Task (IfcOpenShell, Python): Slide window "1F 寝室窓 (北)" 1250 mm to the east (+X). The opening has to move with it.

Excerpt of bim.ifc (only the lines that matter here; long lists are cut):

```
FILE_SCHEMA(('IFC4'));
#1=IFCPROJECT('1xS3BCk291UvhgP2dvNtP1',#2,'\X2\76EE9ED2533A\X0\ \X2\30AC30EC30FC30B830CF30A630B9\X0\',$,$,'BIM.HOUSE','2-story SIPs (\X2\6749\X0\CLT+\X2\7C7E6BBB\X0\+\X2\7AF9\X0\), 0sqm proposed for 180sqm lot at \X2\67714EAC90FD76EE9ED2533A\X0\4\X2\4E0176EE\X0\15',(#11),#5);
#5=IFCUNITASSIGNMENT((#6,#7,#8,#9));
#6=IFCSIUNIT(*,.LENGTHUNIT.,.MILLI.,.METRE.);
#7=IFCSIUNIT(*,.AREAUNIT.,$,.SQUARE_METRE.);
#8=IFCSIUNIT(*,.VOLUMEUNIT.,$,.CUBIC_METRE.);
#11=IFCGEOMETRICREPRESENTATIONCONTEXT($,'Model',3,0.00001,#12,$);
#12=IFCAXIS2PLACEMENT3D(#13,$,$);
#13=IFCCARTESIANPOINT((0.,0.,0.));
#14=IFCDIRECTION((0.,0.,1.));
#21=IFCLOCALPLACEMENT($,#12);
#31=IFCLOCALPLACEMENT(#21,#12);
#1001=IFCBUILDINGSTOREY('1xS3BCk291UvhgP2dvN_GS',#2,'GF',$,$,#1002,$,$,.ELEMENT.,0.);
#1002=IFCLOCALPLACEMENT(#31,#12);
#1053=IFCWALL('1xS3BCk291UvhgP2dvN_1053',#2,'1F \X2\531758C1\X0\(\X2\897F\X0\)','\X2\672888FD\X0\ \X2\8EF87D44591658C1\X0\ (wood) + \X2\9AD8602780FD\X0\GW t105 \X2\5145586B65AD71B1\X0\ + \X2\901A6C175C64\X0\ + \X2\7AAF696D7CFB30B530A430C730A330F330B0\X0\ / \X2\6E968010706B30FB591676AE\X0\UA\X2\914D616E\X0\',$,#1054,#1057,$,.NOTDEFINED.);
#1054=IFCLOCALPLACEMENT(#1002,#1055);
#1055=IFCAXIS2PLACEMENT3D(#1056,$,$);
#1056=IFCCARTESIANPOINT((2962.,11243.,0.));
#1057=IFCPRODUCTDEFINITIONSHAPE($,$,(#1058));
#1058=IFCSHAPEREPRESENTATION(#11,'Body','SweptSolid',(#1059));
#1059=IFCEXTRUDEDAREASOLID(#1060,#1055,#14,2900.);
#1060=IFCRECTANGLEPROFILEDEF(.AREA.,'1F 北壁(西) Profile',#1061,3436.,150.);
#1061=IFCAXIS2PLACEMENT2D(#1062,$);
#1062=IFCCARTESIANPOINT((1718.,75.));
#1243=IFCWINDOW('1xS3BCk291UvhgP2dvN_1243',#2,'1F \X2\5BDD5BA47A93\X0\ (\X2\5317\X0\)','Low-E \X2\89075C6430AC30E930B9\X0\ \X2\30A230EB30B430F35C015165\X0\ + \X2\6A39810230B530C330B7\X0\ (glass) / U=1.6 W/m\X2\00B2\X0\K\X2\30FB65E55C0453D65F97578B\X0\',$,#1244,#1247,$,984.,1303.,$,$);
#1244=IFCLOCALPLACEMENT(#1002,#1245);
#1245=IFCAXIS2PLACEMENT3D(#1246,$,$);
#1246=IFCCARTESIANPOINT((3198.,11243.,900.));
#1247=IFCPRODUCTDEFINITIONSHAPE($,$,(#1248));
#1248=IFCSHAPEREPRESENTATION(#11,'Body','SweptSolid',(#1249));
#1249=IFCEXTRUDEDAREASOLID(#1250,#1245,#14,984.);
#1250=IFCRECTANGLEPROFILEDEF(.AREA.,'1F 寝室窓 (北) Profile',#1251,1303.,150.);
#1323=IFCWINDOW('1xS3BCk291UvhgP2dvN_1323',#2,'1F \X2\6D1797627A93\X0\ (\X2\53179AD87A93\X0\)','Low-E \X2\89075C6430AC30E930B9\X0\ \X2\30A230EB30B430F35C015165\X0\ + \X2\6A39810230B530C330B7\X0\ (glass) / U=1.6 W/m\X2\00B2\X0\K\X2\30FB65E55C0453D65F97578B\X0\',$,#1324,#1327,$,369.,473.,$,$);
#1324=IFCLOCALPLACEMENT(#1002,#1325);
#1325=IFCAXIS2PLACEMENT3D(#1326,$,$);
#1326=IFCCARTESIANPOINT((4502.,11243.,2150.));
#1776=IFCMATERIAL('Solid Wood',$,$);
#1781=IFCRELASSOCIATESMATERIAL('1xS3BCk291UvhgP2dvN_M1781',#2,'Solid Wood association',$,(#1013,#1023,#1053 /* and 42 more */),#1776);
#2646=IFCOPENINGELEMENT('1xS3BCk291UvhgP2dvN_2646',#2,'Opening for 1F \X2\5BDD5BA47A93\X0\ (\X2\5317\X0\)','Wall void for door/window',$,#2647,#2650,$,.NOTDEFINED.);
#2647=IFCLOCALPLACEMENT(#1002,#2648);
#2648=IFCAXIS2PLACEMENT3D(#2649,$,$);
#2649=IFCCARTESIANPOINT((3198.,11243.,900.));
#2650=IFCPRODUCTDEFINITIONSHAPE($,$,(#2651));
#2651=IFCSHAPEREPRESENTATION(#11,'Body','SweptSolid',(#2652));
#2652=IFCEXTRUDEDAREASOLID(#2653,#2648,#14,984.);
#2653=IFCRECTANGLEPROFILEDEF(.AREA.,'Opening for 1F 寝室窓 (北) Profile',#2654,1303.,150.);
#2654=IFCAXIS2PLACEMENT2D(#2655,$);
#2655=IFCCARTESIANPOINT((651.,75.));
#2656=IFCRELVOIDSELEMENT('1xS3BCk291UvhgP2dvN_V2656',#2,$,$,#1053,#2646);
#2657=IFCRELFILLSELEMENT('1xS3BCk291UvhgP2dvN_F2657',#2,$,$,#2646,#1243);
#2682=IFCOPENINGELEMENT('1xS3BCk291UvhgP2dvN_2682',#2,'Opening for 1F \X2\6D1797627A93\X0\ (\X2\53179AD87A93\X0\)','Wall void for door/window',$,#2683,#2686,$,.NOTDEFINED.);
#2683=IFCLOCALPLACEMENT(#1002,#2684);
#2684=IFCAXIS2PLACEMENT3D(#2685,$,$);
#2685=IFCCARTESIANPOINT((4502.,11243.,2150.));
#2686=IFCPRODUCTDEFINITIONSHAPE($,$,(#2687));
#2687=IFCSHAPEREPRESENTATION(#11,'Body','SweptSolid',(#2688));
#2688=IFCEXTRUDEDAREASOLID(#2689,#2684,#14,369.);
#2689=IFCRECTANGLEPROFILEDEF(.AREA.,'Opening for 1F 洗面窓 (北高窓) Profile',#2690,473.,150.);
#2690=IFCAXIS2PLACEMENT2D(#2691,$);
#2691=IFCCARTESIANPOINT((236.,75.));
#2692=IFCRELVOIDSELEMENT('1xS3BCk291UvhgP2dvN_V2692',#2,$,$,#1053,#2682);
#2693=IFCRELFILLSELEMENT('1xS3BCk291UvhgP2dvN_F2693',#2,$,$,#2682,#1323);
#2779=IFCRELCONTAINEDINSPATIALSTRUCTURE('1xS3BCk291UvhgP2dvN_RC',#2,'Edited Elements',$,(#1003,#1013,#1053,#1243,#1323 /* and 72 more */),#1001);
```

```python
import ifcopenshell
import ifcopenshell.api.geometry
import ifcopenshell.util.placement
import ifcopenshell.util.unit

model = ifcopenshell.open("bim.ifc")
unit_scale = ifcopenshell.util.unit.calculate_unit_scale(model)

window = model.by_guid("1xS3BCk291UvhgP2dvN_1243")
opening = window.FillsVoids[0].RelatingOpeningElement
wall = opening.VoidsElements[0].RelatingBuildingElement

wall_matrix = ifcopenshell.util.placement.get_local_placement(wall.ObjectPlacement)
shift = wall_matrix[:3, 0] * 1.25 / unit_scale
before = ifcopenshell.util.placement.get_local_placement(window.ObjectPlacement)[:3, 3].copy()

# The window is not placed relative to its opening, so move both.
for product in (opening, window):
    matrix = ifcopenshell.util.placement.get_local_placement(product.ObjectPlacement)
    matrix[:3, 3] += shift
    ifcopenshell.api.geometry.edit_object_placement(model, product=product, matrix=matrix, is_si=False)

after = ifcopenshell.util.placement.get_local_placement(window.ObjectPlacement)[:3, 3]
print("window moved by", (after - before).round(3) + 0.0)

model.write("bim-out.ifc")
```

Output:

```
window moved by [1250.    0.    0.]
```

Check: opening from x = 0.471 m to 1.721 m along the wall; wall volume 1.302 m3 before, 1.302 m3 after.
